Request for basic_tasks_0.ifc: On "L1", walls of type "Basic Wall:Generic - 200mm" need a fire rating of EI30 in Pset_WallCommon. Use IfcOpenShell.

First a look at what the model holds.

```python
import ifcopenshell
import ifcopenshell.util.element

model = ifcopenshell.open("basic_tasks_0.ifc")
print(model.schema)
storey = next(s for s in model.by_type("IfcBuildingStorey") if s.Name == "L1")
walls = [e for e in ifcopenshell.util.element.get_decomposition(storey) if e.is_a("IfcWall")]
seen = {}
for e in walls:
    element_type = ifcopenshell.util.element.get_type(e)
    key = (element_type.Name if element_type != e and element_type else None, ifcopenshell.util.element.get_pset(e, "Pset_WallCommon", "FireRating"))
    seen[key] = seen.get(key, 0) + 1
for (name, value), count in sorted(seen.items(), key=str):
    print(count, "x", name, "|", value)
```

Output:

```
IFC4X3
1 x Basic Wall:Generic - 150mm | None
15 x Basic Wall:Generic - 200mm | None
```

```python
import ifcopenshell
import ifcopenshell.api.pset
import ifcopenshell.util.element

model = ifcopenshell.open("basic_tasks_0.ifc")

storey = next(s for s in model.by_type("IfcBuildingStorey") if s.Name == "L1")
walls = [e for e in ifcopenshell.util.element.get_decomposition(storey) if e.is_a("IfcWall")]

count = 0
for e in walls:
    element_type = ifcopenshell.util.element.get_type(e)
    if element_type in (None, e) or element_type.Name != "Basic Wall:Generic - 200mm":
        continue
    # add_pset returns the element's existing set when there is one.
    pset = ifcopenshell.api.pset.add_pset(model, product=e, name="Pset_WallCommon")
    ifcopenshell.api.pset.edit_pset(model, pset=pset, properties={"FireRating": "EI30"})
    count += 1

print(count, "walls updated")

model.write("basic_tasks_0-out.ifc")
```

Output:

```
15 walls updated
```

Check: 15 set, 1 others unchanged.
